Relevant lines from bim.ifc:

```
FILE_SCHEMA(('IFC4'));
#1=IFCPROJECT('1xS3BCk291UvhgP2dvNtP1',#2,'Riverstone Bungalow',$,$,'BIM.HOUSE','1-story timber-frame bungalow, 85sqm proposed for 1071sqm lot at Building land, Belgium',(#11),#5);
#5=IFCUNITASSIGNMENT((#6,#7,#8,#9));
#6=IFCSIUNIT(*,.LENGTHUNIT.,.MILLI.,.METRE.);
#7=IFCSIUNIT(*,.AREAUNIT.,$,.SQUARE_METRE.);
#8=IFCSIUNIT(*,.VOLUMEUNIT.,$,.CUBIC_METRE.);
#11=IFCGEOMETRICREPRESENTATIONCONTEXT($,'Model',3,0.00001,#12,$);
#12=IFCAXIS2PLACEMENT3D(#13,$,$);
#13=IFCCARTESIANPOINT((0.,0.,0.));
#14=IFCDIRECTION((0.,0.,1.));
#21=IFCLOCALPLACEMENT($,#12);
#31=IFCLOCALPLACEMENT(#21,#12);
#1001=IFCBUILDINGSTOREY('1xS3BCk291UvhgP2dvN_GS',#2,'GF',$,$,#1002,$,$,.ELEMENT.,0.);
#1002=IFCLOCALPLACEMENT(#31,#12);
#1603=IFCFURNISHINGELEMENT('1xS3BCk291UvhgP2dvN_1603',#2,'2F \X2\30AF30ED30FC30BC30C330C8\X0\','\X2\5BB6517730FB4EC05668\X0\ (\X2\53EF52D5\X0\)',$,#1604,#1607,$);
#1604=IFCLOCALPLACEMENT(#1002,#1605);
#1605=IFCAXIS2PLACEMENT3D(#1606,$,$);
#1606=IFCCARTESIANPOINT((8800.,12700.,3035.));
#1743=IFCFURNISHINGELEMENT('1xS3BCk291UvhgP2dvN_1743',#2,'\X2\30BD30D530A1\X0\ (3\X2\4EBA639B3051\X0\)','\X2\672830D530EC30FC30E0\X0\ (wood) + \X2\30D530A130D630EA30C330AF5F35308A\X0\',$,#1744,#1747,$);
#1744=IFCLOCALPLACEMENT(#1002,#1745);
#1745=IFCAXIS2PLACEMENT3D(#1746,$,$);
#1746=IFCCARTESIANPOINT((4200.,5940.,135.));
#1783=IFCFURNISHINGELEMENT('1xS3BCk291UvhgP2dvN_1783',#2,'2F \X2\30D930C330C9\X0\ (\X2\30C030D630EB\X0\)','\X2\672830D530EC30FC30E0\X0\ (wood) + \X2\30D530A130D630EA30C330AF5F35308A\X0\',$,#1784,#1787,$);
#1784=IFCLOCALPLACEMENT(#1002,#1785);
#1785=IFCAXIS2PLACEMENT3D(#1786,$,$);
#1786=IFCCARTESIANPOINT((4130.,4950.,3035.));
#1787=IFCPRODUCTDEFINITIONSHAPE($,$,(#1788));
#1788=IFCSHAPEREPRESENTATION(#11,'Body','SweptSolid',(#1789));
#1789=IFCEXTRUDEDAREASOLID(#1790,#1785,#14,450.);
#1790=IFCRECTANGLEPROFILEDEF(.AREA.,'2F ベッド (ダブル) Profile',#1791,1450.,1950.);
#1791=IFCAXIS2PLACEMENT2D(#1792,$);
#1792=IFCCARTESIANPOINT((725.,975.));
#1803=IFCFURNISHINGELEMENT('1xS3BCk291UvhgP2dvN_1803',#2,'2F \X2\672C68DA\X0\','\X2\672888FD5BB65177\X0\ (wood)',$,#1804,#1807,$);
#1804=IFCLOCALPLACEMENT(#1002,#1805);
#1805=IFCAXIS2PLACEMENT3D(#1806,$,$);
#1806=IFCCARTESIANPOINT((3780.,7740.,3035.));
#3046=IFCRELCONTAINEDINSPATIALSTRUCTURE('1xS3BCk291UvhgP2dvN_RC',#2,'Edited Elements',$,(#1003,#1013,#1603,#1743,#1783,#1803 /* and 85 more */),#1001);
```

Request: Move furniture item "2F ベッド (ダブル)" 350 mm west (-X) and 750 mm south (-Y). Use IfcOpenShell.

```python
import ifcopenshell
import ifcopenshell.api.geometry
import ifcopenshell.util.placement
import ifcopenshell.util.unit

model = ifcopenshell.open("bim.ifc")
unit_scale = ifcopenshell.util.unit.calculate_unit_scale(model)

item = model.by_guid("1xS3BCk291UvhgP2dvN_1783")
matrix = ifcopenshell.util.placement.get_local_placement(item.ObjectPlacement)
matrix[0, 3] -= 0.35 / unit_scale
matrix[1, 3] -= 0.75 / unit_scale
ifcopenshell.api.geometry.edit_object_placement(model, product=item, matrix=matrix, is_si=False)

print(ifcopenshell.util.placement.get_local_placement(item.ObjectPlacement).round(3) + 0.0)

model.write("bim_rev.ifc")
```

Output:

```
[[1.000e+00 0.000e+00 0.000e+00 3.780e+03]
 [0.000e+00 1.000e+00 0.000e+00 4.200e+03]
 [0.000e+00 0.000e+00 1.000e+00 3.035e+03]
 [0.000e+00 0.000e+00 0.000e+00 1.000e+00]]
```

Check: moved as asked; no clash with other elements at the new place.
